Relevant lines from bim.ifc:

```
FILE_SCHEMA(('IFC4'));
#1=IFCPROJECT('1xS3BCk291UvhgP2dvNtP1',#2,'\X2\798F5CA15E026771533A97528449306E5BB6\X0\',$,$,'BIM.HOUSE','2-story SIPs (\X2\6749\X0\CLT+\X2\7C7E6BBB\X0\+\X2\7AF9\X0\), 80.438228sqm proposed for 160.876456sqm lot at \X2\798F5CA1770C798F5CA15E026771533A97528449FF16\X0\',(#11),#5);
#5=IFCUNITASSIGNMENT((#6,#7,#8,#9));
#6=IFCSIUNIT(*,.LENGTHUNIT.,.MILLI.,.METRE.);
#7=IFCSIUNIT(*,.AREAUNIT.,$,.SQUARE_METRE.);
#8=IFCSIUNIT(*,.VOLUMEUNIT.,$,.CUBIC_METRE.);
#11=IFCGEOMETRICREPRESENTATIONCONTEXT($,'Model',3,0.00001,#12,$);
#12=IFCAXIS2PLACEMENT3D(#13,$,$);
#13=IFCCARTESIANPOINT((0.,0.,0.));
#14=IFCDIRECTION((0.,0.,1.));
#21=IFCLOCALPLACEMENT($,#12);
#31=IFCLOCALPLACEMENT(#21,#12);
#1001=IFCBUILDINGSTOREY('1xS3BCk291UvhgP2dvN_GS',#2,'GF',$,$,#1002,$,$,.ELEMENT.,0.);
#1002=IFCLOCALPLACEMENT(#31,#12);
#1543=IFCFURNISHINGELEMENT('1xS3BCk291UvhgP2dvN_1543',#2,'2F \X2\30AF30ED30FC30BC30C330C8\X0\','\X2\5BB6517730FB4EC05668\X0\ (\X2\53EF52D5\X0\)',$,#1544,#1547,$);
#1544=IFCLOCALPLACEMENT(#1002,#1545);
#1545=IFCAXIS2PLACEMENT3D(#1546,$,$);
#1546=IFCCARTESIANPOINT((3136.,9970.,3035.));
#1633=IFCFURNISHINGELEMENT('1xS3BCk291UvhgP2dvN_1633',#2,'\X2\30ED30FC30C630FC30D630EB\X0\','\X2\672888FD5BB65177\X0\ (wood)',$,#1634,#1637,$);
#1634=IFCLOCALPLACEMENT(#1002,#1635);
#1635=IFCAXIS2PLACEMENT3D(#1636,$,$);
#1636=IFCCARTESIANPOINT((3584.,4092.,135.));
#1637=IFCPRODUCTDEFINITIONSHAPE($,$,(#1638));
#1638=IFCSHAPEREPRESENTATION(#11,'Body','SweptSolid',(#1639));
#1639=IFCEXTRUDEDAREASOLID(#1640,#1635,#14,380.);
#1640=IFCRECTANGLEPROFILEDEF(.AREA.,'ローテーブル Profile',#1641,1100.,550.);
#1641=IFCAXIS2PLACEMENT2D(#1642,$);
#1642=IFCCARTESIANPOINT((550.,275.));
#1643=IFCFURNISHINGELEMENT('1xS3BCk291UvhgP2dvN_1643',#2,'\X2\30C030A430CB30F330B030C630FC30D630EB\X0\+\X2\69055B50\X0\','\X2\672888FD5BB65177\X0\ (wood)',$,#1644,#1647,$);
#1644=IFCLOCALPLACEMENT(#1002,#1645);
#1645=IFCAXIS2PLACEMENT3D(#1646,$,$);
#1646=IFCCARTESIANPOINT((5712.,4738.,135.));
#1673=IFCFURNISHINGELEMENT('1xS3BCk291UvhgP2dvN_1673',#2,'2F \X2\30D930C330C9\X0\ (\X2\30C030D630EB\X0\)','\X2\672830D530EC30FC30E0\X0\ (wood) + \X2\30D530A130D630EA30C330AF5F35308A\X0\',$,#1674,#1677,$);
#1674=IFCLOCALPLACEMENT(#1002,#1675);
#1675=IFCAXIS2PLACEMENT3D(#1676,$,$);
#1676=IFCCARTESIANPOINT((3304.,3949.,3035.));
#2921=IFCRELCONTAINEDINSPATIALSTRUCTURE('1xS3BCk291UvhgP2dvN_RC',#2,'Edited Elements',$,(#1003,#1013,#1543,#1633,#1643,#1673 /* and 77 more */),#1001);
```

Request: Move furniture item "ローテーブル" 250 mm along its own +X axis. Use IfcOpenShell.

```python
import ifcopenshell
import ifcopenshell.api.geometry
import ifcopenshell.util.placement

model = ifcopenshell.open("bim.ifc")

item = model.by_guid("1xS3BCk291UvhgP2dvN_1633")
matrix = ifcopenshell.util.placement.get_local_placement(item.ObjectPlacement)
matrix[:3, 3] += matrix[:3, 0] * 250.0
ifcopenshell.api.geometry.edit_object_placement(model, product=item, matrix=matrix, is_si=False)

print(ifcopenshell.util.placement.get_local_placement(item.ObjectPlacement).round(3) + 0.0)

model.write("bim_edited.ifc")
```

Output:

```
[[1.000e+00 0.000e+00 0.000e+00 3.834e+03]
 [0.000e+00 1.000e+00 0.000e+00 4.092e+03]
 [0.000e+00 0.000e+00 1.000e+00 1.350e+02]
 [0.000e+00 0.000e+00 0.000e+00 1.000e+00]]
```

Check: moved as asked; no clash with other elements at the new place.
